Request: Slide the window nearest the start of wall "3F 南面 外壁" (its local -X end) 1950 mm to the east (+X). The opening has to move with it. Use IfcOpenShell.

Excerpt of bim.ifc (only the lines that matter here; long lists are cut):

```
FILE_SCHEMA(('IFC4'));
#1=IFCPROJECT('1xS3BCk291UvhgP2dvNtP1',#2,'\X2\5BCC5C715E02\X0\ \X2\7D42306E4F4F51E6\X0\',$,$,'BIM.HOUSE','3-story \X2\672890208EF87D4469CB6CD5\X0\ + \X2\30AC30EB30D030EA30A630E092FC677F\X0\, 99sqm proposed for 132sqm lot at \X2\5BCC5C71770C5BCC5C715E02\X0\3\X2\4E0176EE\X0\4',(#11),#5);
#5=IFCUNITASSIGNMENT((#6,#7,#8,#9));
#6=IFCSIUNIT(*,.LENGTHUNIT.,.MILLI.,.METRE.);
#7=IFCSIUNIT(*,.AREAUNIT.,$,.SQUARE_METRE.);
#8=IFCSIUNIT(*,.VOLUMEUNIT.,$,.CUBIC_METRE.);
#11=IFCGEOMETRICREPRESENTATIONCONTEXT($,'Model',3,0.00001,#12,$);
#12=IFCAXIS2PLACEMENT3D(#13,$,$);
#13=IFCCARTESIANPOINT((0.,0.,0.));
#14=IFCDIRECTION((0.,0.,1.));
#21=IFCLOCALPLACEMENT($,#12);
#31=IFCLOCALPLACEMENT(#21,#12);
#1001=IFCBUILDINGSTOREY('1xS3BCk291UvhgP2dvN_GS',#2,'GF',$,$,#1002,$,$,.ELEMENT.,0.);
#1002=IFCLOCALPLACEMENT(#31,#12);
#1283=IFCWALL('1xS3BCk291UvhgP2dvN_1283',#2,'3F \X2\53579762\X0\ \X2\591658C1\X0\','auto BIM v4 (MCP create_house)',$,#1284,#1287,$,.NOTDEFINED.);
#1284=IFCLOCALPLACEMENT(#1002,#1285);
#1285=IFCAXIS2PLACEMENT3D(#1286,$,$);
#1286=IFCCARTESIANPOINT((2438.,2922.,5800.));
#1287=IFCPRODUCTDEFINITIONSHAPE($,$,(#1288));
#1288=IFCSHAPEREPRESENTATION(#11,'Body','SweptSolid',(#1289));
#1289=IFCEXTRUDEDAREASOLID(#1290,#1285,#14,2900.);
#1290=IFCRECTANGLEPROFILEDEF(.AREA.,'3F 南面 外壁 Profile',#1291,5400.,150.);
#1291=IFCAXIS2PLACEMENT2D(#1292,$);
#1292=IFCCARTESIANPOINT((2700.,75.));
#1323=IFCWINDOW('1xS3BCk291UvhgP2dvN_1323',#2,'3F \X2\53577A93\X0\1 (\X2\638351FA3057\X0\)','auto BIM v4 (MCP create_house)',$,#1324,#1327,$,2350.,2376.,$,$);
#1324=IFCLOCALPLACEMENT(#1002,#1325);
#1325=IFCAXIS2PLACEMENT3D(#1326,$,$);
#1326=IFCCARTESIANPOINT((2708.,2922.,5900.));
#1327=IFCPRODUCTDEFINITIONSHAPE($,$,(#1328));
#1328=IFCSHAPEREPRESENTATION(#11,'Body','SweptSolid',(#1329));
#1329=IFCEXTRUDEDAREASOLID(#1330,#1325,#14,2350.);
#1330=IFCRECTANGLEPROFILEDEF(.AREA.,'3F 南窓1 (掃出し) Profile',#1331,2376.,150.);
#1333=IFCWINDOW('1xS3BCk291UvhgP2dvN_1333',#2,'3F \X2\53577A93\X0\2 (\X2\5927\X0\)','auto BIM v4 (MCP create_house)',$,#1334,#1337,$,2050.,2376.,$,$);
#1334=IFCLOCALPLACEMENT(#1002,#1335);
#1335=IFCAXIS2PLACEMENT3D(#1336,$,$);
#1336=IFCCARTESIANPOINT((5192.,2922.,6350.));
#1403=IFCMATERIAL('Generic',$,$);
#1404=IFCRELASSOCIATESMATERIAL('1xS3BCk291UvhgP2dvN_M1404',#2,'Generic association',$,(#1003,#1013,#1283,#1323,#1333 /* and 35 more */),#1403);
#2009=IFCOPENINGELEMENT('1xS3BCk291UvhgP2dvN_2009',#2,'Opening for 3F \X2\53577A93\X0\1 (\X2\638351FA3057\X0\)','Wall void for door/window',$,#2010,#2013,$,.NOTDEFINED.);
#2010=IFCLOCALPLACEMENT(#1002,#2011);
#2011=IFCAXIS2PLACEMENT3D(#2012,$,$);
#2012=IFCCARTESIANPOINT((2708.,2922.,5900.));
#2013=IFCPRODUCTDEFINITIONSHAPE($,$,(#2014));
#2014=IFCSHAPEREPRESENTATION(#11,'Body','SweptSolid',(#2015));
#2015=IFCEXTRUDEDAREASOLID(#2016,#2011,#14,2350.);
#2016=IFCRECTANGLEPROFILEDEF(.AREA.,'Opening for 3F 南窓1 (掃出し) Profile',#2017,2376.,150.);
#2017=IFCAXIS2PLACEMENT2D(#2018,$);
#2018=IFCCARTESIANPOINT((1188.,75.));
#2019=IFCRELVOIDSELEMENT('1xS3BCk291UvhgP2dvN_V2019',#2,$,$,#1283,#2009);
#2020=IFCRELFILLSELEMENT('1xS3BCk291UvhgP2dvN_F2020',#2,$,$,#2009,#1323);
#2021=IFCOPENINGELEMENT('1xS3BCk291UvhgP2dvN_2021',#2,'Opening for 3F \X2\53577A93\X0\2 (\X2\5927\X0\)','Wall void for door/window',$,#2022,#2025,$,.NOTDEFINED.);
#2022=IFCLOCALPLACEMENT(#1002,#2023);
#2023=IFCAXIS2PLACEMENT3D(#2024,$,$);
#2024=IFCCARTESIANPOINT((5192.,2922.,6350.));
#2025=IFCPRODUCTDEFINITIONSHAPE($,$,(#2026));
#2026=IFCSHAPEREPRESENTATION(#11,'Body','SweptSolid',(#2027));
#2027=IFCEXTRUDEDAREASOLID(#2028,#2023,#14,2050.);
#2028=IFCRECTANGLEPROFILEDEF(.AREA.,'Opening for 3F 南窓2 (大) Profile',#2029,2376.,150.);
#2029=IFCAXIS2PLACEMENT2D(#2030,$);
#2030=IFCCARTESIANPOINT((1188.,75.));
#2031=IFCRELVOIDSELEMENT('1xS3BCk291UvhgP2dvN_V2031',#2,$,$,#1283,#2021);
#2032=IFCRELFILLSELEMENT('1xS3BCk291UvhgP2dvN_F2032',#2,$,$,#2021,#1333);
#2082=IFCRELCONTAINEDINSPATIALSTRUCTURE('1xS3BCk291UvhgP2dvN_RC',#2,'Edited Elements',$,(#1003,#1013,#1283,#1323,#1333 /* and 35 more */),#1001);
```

```python
import ifcopenshell
import ifcopenshell.api.geometry
import ifcopenshell.util.placement

model = ifcopenshell.open("bim.ifc")

window = model.by_guid("1xS3BCk291UvhgP2dvN_1323")
opening = window.FillsVoids[0].RelatingOpeningElement
wall = opening.VoidsElements[0].RelatingBuildingElement

wall_matrix = ifcopenshell.util.placement.get_local_placement(wall.ObjectPlacement)
shift = wall_matrix[:3, 0] * 1950.0
before = ifcopenshell.util.placement.get_local_placement(window.ObjectPlacement)[:3, 3].copy()

# The window is not placed relative to its opening, so move both.
for product in (opening, window):
    matrix = ifcopenshell.util.placement.get_local_placement(product.ObjectPlacement)
    matrix[:3, 3] += shift
    ifcopenshell.api.geometry.edit_object_placement(model, product=product, matrix=matrix, is_si=False)

after = ifcopenshell.util.placement.get_local_placement(window.ObjectPlacement)[:3, 3]
print("window moved by", (after - before).round(3) + 0.0)

model.write("bim-out.ifc")
```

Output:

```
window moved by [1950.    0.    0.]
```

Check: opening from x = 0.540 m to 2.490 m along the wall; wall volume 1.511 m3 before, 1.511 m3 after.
